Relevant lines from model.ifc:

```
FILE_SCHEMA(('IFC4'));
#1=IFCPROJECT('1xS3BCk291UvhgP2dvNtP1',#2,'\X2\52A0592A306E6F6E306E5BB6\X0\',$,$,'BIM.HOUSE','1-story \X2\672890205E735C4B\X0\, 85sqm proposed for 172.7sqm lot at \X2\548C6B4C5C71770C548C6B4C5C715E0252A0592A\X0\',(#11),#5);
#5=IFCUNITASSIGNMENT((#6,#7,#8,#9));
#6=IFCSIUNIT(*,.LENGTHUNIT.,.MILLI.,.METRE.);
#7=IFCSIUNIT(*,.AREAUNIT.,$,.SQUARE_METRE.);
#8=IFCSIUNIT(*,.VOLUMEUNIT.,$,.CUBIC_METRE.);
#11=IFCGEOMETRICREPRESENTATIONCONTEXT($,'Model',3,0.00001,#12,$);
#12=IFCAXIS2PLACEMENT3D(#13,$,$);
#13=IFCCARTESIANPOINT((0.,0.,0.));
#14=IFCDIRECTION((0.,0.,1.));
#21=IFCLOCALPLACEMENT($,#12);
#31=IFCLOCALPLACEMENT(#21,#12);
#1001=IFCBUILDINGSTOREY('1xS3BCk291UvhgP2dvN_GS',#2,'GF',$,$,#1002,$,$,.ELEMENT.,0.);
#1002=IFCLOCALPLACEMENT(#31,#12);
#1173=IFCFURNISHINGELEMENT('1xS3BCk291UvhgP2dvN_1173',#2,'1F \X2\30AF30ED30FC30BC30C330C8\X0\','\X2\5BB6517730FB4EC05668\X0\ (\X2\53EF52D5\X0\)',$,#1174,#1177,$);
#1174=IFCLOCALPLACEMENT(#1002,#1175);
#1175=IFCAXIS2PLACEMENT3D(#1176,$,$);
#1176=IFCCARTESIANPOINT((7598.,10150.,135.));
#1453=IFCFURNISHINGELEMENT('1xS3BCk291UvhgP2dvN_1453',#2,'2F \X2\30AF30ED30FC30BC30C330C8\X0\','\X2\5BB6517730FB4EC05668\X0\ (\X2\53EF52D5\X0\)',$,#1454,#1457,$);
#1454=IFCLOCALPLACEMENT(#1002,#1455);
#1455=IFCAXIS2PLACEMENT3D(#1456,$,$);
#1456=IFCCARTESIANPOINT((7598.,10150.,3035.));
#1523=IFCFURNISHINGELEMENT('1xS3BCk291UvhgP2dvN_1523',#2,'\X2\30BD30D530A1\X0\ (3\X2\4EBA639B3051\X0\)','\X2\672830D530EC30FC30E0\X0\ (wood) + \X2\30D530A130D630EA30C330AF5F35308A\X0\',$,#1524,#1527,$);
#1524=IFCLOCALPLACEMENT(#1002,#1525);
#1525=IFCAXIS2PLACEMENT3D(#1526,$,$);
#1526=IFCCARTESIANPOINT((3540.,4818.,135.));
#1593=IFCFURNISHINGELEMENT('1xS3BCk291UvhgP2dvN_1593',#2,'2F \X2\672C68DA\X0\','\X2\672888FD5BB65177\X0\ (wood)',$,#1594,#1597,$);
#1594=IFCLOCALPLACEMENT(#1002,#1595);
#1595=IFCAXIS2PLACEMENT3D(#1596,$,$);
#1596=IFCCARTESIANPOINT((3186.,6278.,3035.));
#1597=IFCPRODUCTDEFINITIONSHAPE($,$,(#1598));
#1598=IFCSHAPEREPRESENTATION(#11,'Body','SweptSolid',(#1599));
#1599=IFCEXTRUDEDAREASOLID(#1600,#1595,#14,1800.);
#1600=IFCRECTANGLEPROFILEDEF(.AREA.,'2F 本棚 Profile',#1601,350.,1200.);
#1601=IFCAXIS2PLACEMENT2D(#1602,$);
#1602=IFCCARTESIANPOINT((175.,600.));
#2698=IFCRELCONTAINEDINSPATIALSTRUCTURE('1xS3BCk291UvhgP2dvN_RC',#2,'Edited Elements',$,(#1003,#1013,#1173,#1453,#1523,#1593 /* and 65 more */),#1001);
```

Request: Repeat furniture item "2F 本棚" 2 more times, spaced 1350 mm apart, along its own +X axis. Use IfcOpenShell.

```python
import ifcopenshell
import ifcopenshell.api.geometry
import ifcopenshell.api.root
import ifcopenshell.util.element
import ifcopenshell.util.placement
import ifcopenshell.util.unit

model = ifcopenshell.open("model.ifc")
unit_scale = ifcopenshell.util.unit.calculate_unit_scale(model)


def reuse_history(source, copy):
    """copy_class also copies each property set's owner history, people and application; keep the originals."""
    for rel in copy.IsDefinedBy:
        if rel.is_a("IfcRelDefinesByProperties") and (history := rel.RelatingPropertyDefinition.OwnerHistory):
            rel.RelatingPropertyDefinition.OwnerHistory = source.OwnerHistory
            ifcopenshell.util.element.remove_deep2(model, history)


source = model.by_guid("1xS3BCk291UvhgP2dvN_1593")
base = ifcopenshell.util.placement.get_local_placement(source.ObjectPlacement)
step = base[:3, 0] * 1.35 / unit_scale

for i in range(1, 3):
    copy = ifcopenshell.api.root.copy_class(model, product=source)
    copy.Representation = ifcopenshell.util.element.copy_deep(
        model, source.Representation, exclude=["IfcGeometricRepresentationContext", "IfcRepresentationMap"]
    )
    reuse_history(source, copy)
    matrix = base.copy()
    matrix[:3, 3] += i * step
    print("added at", matrix[:3, 3].round(3) + 0.0)
    ifcopenshell.api.geometry.edit_object_placement(model, product=copy, matrix=matrix, is_si=False)

model.write("model_updated.ifc")
```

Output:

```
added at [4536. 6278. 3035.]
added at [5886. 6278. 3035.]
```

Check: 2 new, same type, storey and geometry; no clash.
